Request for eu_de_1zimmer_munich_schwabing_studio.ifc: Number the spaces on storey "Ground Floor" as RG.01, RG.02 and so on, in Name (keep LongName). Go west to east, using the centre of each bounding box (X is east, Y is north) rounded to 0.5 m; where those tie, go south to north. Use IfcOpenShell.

First a look at what the model holds.

```python
import ifcopenshell
import ifcopenshell.util.element
import ifcopenshell.util.placement

model = ifcopenshell.open("eu_de_1zimmer_munich_schwabing_studio.ifc")
print(model.schema)
storey = next(s for s in model.by_type("IfcBuildingStorey") if s.Name == "Ground Floor")
spaces = [e for e in ifcopenshell.util.element.get_decomposition(storey) if e.is_a("IfcSpace")]
for e in sorted(spaces, key=lambda e: e.id()):
    origin = ifcopenshell.util.placement.get_local_placement(e.ObjectPlacement)[:3, 3]
    print(e.id(), e.Name, e.LongName, origin.round(2) + 0.0, sep=" | ")
```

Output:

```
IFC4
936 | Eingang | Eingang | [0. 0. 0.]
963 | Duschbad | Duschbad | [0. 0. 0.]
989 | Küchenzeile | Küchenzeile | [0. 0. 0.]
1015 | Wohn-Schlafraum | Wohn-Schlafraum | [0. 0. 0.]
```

```python
import ifcopenshell
import ifcopenshell.geom
import ifcopenshell.util.element
import ifcopenshell.util.shape

model = ifcopenshell.open("eu_de_1zimmer_munich_schwabing_studio.ifc")
settings = ifcopenshell.geom.settings()
settings.set("use-world-coords", True)


def centre(element):
    shape = ifcopenshell.geom.create_shape(settings, element)
    return ifcopenshell.util.shape.get_bbox_centroid(shape.geometry)


storey = next(s for s in model.by_type("IfcBuildingStorey") if s.Name == "Ground Floor")
spaces = [e for e in ifcopenshell.util.element.get_decomposition(storey) if e.is_a("IfcSpace")]

# Insertion points can sit at a corner or the storey origin, so sort by the geometry (in metres).
centres = {e: centre(e) for e in spaces}
spaces.sort(key=lambda e: (round(centres[e][0] / 0.5), centres[e][1]))

for i, e in enumerate(spaces, start=1):
    number = f"RG.{i:02d}"
    e.Name = number
    print(e.id(), number)

model.write("eu_de_1zimmer_munich_schwabing_studio_v2.ifc")
```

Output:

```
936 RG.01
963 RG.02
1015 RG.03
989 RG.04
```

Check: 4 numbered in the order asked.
